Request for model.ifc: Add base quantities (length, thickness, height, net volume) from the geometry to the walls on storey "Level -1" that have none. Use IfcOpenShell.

First a look at what the model holds.

```python
import ifcopenshell
import ifcopenshell.util.element
import ifcopenshell.util.unit

model = ifcopenshell.open("model.ifc")
print(model.schema)
for unit_type in ("LENGTHUNIT", "AREAUNIT", "VOLUMEUNIT"):
    print(unit_type, ifcopenshell.util.unit.calculate_unit_scale(model, unit_type))
storey = next(s for s in model.by_type("IfcBuildingStorey") if s.Name == "Level -1")
walls = [e for e in ifcopenshell.util.element.get_decomposition(storey) if e.is_a("IfcWall")]
for e in sorted(walls, key=lambda e: e.id()):
    print(e.id(), e.is_a(), e.Name, list(ifcopenshell.util.element.get_psets(e, qtos_only=True)), sep=" | ")
```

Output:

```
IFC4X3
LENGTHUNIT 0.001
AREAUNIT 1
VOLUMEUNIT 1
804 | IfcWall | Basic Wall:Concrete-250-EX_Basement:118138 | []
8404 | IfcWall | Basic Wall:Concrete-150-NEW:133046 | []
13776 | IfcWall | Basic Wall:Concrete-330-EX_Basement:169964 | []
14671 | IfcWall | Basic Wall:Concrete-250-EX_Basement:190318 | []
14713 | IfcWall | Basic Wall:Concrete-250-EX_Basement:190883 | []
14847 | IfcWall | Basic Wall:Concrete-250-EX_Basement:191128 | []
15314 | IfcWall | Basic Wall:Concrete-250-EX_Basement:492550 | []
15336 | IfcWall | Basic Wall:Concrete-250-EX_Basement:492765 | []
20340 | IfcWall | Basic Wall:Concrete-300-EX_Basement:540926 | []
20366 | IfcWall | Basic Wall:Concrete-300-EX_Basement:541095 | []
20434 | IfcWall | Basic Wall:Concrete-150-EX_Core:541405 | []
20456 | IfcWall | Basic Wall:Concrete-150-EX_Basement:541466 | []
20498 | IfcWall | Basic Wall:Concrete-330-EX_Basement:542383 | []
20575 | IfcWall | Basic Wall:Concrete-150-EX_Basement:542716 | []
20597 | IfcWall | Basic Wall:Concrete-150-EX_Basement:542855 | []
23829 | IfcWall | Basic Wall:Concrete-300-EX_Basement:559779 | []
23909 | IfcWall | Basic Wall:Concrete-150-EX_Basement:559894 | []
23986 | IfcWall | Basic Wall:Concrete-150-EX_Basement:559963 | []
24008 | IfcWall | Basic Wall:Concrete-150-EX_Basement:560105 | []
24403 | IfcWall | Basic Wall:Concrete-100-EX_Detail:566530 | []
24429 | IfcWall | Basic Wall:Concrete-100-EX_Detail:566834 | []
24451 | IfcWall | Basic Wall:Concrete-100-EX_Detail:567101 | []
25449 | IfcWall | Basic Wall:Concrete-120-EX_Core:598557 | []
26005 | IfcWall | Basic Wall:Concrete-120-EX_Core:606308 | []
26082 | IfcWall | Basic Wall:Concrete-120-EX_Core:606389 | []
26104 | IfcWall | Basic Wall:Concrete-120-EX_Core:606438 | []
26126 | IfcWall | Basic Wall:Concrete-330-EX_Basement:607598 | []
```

```python
import ifcopenshell
import ifcopenshell.api.pset
import ifcopenshell.geom
import ifcopenshell.util.element
import ifcopenshell.util.shape
import ifcopenshell.util.unit

model = ifcopenshell.open("model.ifc")
unit_scale = ifcopenshell.util.unit.calculate_unit_scale(model)
volume_scale = ifcopenshell.util.unit.calculate_unit_scale(model, "VOLUMEUNIT")
settings = ifcopenshell.geom.settings()

storey = next(s for s in model.by_type("IfcBuildingStorey") if s.Name == "Level -1")
walls = [e for e in ifcopenshell.util.element.get_decomposition(storey) if e.is_a("IfcWall")]

for e in sorted(walls, key=lambda e: e.id()):
    if ifcopenshell.util.element.get_psets(e, qtos_only=True, should_inherit=False):
        continue
    # Geometry comes back in metres, in the element's own axes.
    shape = ifcopenshell.geom.create_shape(settings, e)
    values = {
        "Length": ifcopenshell.util.shape.get_x(shape.geometry) / unit_scale,
        "Width": ifcopenshell.util.shape.get_y(shape.geometry) / unit_scale,
        "Height": ifcopenshell.util.shape.get_z(shape.geometry) / unit_scale,
        "NetVolume": ifcopenshell.util.shape.get_volume(shape.geometry) / volume_scale,
    }
    qto = ifcopenshell.api.pset.add_qto(model, product=e, name="Qto_WallBaseQuantities")
    ifcopenshell.api.pset.edit_qto(model, qto=qto, properties=values)
    print(e.id(), {k: round(v, 3) for k, v in values.items()})

model.write("model_v2.ifc")
```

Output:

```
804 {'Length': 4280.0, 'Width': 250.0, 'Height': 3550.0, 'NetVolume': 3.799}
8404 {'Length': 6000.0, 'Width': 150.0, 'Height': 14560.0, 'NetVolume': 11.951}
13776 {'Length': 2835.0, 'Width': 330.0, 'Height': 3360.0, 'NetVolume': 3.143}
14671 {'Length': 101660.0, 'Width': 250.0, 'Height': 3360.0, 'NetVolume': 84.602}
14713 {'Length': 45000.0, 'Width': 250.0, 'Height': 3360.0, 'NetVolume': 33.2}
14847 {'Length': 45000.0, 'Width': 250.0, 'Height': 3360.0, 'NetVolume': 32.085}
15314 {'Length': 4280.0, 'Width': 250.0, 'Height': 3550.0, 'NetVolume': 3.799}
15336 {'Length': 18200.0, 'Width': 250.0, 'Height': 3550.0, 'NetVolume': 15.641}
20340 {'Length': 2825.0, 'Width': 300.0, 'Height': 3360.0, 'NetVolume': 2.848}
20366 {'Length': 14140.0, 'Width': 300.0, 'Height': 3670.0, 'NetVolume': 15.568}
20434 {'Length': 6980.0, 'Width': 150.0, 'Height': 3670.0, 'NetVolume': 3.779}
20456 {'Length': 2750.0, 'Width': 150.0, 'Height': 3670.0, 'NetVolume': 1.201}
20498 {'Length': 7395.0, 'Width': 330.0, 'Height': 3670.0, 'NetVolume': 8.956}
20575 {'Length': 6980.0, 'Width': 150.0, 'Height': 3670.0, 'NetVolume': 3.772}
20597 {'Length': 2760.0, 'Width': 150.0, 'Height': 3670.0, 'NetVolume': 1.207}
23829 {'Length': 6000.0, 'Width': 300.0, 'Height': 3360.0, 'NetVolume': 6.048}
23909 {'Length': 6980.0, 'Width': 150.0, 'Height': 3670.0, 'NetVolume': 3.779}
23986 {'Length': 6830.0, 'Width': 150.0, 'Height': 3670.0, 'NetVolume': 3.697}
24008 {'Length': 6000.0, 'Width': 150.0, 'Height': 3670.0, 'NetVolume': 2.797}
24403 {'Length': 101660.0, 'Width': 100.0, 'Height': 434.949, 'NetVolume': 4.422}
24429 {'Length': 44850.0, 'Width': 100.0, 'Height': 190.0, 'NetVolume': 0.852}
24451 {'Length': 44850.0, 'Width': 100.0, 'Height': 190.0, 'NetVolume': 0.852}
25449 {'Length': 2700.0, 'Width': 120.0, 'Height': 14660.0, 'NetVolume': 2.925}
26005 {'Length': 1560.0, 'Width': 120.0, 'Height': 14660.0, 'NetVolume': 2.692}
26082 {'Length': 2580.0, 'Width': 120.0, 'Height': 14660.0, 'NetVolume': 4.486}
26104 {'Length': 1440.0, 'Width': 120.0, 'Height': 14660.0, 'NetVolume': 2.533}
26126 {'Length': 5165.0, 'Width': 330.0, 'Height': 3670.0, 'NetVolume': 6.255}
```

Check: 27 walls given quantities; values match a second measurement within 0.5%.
